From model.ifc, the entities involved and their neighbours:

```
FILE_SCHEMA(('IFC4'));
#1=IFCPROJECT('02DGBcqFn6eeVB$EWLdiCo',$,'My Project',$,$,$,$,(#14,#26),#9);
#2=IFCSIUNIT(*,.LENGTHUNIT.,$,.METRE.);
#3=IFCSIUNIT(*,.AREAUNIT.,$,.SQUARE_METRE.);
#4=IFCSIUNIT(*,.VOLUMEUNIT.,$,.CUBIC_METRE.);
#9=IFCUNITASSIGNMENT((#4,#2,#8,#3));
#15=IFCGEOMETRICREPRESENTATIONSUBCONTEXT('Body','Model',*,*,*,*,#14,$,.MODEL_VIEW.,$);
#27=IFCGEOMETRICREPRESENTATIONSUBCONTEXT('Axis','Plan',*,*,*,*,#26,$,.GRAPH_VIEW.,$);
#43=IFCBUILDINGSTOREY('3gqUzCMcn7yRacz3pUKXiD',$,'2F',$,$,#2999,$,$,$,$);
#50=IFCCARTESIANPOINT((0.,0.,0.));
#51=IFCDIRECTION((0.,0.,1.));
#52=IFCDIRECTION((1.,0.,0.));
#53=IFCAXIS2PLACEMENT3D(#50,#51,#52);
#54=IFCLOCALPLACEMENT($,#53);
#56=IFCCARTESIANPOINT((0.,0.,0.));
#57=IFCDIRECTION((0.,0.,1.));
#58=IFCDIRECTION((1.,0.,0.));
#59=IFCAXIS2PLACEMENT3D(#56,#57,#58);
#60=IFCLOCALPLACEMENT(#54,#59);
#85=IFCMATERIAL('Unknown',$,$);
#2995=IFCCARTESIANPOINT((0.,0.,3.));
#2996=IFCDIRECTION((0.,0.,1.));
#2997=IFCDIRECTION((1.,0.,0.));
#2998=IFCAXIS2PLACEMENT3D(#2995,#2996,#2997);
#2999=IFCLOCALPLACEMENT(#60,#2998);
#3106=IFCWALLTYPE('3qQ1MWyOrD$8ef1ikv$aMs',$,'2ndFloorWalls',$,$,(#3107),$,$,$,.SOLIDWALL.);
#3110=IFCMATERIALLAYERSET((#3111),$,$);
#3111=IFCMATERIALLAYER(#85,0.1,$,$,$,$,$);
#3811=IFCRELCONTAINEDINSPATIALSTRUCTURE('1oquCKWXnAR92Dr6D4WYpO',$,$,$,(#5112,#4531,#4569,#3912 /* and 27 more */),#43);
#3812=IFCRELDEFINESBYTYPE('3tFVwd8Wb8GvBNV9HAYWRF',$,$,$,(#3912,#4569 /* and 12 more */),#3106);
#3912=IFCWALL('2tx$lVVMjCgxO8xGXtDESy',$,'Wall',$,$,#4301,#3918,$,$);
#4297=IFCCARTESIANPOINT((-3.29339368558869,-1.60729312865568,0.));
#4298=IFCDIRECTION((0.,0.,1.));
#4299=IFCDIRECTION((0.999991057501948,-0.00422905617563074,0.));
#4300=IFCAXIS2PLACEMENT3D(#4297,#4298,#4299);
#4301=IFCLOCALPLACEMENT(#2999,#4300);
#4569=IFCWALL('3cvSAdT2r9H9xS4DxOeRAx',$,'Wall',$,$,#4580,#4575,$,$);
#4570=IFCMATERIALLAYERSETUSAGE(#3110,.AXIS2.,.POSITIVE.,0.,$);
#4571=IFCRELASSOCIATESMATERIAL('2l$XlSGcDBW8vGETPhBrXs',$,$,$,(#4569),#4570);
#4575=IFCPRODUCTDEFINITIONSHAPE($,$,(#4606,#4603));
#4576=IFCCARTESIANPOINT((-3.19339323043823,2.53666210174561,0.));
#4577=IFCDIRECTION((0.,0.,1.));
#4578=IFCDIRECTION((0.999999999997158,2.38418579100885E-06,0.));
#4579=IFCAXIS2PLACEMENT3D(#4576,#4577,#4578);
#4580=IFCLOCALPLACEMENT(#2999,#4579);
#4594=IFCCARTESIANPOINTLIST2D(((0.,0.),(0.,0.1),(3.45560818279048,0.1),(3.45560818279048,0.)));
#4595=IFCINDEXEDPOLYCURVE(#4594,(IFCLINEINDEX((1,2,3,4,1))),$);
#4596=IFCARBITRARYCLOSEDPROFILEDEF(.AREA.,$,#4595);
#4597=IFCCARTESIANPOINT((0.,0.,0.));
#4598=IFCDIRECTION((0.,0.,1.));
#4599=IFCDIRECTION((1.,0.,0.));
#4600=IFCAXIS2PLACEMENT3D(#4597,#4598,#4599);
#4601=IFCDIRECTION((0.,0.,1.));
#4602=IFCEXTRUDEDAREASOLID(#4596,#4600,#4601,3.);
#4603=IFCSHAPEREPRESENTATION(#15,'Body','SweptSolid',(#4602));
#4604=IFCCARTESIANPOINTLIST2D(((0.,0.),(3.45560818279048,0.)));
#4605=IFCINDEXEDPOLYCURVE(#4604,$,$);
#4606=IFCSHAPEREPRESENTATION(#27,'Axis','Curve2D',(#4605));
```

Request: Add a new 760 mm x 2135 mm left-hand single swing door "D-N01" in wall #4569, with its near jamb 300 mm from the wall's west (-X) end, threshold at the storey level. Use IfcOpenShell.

```python
import numpy as np
import ifcopenshell
import ifcopenshell.api.feature
import ifcopenshell.api.geometry
import ifcopenshell.api.root
import ifcopenshell.api.spatial
import ifcopenshell.geom
import ifcopenshell.util.element
import ifcopenshell.util.placement
import ifcopenshell.util.representation
import ifcopenshell.util.shape
import ifcopenshell.util.unit

model = ifcopenshell.open("model.ifc")
unit_scale = ifcopenshell.util.unit.calculate_unit_scale(model)
settings = ifcopenshell.geom.settings()


def volume(element):
    """Net volume in cubic metres, openings subtracted."""
    shape = ifcopenshell.geom.create_shape(settings, element)
    return ifcopenshell.util.shape.get_volume(shape.geometry)


wall = model.by_guid("3cvSAdT2r9H9xS4DxOeRAx")
storey = ifcopenshell.util.element.get_container(wall, ifc_class="IfcBuildingStorey")
context = ifcopenshell.util.representation.get_context(model, "Model", "Body", "MODEL_VIEW")
before = volume(wall)

width, height, from_end, sill = 0.76, 2.135, 0.3, 0.0  # metres

# The wall runs along its own X axis, and the end named is its -X end.
wall_shape = ifcopenshell.geom.create_shape(settings, wall)
x, y, z = ifcopenshell.util.shape.get_vertices(wall_shape.geometry).T
start = x.min() + from_end
face, thickness = float(y.min()), float(y.max() - y.min())
wall_matrix = ifcopenshell.util.placement.get_local_placement(wall.ObjectPlacement)
level = ifcopenshell.util.placement.get_local_placement(storey.ObjectPlacement)[2, 3]


def in_wall(x, y):
    """Placement at x, y metres in the wall's axes, at sill height."""
    matrix = wall_matrix.copy()
    matrix[:, 3] = wall_matrix @ np.array([x / unit_scale, y / unit_scale, 0.0, 1.0])
    matrix[2, 3] = level + sill / unit_scale
    return matrix


# Opening: a box that overshoots both wall faces by 50 mm.
opening = ifcopenshell.api.root.create_entity(model, ifc_class="IfcOpeningElement", predefined_type="OPENING")
box = ifcopenshell.api.geometry.add_wall_representation(
    model, context=context, length=width, height=height, thickness=thickness + 0.1
)
ifcopenshell.api.geometry.assign_representation(model, product=opening, representation=box)
ifcopenshell.api.geometry.edit_object_placement(model, product=opening, matrix=in_wall(start, face - 0.05), is_si=False)
ifcopenshell.api.feature.add_feature(model, feature=opening, element=wall)

door = ifcopenshell.api.root.create_entity(model, ifc_class="IfcDoor", name="D-N01", predefined_type="DOOR")
door.OverallWidth, door.OverallHeight = width / unit_scale, height / unit_scale
door.OperationType = "SINGLE_SWING_LEFT"
body = ifcopenshell.api.geometry.add_door_representation(
    model,
    context=context,
    overall_width=door.OverallWidth,
    overall_height=door.OverallHeight,
    operation_type="SINGLE_SWING_LEFT",
    lining_properties={"LiningDepth": thickness / unit_scale, "ThresholdDepth": thickness / unit_scale},
)
ifcopenshell.api.geometry.assign_representation(model, product=door, representation=body)
ifcopenshell.api.spatial.assign_container(model, products=[door], relating_structure=storey)
ifcopenshell.api.feature.add_filling(model, opening=opening, element=door)

# The lining spans the wall, so the door starts at the wall face.
ifcopenshell.api.geometry.edit_object_placement(model, product=door, matrix=in_wall(start, face), is_si=False)

after = volume(wall)

print(f"wall volume {before:.3f} -> {after:.3f} m3")

model.write("model_updated.ifc")
```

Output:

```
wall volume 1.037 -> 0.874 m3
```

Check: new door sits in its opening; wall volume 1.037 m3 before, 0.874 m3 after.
